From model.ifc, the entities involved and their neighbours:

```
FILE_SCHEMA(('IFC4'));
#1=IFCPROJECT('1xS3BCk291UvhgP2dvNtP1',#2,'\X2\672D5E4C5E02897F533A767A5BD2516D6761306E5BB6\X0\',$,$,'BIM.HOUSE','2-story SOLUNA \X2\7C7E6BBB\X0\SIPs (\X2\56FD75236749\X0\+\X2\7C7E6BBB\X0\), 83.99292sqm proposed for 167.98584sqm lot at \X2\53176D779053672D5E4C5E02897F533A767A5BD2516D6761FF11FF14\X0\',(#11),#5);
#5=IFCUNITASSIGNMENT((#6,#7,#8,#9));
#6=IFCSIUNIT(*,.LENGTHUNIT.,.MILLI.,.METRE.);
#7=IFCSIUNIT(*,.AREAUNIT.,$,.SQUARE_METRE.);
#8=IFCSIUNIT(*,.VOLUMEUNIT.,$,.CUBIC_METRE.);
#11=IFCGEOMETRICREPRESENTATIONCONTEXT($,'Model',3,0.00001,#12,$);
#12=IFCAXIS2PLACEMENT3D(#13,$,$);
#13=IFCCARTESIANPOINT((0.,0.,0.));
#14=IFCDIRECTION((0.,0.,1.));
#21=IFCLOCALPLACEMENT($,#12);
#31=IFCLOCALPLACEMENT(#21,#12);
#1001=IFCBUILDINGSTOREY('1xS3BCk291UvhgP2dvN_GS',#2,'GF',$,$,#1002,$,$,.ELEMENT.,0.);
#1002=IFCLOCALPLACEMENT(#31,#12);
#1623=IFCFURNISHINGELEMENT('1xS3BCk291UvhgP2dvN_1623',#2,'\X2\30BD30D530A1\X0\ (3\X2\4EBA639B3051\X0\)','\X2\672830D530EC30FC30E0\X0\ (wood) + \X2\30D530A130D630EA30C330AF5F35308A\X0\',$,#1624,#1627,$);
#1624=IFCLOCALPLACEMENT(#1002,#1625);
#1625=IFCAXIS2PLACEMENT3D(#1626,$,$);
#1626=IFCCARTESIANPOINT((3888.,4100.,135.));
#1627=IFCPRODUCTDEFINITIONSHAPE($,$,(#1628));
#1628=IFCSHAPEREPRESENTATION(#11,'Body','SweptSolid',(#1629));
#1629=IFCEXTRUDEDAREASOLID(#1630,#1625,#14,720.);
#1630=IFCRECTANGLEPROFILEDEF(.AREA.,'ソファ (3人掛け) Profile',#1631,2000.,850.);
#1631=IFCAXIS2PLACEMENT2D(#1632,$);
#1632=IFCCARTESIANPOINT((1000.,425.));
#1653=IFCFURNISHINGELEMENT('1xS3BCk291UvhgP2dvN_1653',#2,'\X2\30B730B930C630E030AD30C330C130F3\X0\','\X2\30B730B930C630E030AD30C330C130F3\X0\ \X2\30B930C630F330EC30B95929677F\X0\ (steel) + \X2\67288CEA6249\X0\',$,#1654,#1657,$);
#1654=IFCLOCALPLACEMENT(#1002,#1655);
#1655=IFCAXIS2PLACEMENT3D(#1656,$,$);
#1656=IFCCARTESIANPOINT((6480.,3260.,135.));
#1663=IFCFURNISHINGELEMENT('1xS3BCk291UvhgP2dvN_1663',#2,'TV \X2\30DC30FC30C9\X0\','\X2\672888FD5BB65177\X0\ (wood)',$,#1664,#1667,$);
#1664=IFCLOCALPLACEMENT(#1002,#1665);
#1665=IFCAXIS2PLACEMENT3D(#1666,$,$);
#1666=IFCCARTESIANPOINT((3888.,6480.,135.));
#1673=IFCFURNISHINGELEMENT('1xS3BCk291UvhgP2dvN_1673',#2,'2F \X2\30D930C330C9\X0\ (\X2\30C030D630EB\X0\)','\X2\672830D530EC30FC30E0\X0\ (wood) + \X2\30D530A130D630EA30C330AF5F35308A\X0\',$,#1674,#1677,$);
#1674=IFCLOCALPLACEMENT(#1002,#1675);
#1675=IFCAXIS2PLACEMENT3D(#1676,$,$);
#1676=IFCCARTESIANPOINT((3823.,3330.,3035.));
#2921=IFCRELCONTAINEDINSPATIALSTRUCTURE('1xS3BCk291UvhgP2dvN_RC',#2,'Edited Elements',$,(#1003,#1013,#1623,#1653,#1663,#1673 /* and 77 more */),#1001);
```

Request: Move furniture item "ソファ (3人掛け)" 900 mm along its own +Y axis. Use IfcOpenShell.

```python
import ifcopenshell
import ifcopenshell.api.geometry
import ifcopenshell.util.placement
import ifcopenshell.util.unit

model = ifcopenshell.open("model.ifc")
unit_scale = ifcopenshell.util.unit.calculate_unit_scale(model)

item = model.by_guid("1xS3BCk291UvhgP2dvN_1623")
matrix = ifcopenshell.util.placement.get_local_placement(item.ObjectPlacement)
matrix[:3, 3] += matrix[:3, 1] * 0.9 / unit_scale
ifcopenshell.api.geometry.edit_object_placement(model, product=item, matrix=matrix, is_si=False)

print(ifcopenshell.util.placement.get_local_placement(item.ObjectPlacement).round(3) + 0.0)

model.write("model-out.ifc")
```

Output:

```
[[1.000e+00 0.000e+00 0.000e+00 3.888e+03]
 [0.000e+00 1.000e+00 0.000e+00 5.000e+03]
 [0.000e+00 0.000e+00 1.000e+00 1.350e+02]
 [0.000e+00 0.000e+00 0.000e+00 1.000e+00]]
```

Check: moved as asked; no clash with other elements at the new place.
